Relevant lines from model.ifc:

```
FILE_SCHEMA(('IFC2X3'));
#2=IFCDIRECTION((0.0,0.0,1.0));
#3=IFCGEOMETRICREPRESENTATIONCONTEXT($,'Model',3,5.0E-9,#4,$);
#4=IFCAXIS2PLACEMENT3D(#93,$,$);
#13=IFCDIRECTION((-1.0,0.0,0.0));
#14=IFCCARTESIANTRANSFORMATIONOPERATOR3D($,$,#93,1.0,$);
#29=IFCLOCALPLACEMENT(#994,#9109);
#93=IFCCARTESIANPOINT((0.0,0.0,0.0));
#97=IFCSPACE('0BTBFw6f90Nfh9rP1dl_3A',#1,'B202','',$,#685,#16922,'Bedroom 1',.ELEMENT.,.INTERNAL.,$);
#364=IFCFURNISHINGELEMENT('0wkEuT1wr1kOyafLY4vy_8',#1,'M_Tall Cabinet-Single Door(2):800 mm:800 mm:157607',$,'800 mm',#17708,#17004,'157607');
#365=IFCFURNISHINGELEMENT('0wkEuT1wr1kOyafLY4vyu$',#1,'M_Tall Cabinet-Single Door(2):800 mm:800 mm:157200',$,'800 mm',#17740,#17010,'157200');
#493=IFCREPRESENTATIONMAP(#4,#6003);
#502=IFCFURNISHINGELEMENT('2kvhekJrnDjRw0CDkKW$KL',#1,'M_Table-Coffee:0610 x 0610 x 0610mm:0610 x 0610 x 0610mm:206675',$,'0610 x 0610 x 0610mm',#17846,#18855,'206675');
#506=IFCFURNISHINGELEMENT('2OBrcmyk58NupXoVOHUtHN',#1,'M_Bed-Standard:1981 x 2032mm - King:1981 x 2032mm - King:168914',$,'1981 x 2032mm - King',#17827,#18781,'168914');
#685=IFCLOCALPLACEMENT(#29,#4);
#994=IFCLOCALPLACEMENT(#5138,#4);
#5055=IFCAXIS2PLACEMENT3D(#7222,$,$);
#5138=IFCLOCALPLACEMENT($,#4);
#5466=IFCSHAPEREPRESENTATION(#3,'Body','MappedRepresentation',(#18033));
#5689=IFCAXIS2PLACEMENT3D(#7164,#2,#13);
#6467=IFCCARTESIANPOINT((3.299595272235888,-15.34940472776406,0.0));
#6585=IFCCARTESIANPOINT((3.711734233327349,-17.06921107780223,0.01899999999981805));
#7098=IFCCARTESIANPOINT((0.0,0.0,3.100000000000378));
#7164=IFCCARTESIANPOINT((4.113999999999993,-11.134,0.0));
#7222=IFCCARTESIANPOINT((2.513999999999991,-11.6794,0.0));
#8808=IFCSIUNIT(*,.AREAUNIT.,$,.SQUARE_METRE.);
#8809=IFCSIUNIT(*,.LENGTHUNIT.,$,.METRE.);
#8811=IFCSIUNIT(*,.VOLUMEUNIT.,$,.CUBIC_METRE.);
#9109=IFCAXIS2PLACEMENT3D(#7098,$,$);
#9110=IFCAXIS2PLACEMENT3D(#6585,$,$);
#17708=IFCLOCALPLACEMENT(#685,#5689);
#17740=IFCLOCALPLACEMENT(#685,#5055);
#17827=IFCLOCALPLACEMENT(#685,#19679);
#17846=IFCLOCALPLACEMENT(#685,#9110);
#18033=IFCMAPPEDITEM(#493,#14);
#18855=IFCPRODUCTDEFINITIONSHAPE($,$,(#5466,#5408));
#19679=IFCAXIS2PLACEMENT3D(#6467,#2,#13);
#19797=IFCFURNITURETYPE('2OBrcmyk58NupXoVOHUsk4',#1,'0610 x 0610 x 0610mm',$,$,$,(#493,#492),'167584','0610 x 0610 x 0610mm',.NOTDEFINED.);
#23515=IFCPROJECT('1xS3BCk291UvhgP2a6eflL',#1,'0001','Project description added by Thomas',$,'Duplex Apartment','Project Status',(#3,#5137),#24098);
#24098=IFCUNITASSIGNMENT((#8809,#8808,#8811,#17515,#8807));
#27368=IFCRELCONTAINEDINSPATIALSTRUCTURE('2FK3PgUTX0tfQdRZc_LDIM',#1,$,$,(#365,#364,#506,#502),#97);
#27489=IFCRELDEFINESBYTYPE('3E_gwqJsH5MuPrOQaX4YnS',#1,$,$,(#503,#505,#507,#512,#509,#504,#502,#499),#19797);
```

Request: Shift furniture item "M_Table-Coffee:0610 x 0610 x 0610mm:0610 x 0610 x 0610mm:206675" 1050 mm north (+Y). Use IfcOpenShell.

```python
import ifcopenshell
import ifcopenshell.api.geometry
import ifcopenshell.util.placement
import ifcopenshell.util.unit

model = ifcopenshell.open("model.ifc")
unit_scale = ifcopenshell.util.unit.calculate_unit_scale(model)

item = model.by_id(502)
matrix = ifcopenshell.util.placement.get_local_placement(item.ObjectPlacement)
matrix[1, 3] += 1.05 / unit_scale
ifcopenshell.api.geometry.edit_object_placement(model, product=item, matrix=matrix, is_si=False)

print(ifcopenshell.util.placement.get_local_placement(item.ObjectPlacement).round(3) + 0.0)

model.write("model_rev.ifc")
```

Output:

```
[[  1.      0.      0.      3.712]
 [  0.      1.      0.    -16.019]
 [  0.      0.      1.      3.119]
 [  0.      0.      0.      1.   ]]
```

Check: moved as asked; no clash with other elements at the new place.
